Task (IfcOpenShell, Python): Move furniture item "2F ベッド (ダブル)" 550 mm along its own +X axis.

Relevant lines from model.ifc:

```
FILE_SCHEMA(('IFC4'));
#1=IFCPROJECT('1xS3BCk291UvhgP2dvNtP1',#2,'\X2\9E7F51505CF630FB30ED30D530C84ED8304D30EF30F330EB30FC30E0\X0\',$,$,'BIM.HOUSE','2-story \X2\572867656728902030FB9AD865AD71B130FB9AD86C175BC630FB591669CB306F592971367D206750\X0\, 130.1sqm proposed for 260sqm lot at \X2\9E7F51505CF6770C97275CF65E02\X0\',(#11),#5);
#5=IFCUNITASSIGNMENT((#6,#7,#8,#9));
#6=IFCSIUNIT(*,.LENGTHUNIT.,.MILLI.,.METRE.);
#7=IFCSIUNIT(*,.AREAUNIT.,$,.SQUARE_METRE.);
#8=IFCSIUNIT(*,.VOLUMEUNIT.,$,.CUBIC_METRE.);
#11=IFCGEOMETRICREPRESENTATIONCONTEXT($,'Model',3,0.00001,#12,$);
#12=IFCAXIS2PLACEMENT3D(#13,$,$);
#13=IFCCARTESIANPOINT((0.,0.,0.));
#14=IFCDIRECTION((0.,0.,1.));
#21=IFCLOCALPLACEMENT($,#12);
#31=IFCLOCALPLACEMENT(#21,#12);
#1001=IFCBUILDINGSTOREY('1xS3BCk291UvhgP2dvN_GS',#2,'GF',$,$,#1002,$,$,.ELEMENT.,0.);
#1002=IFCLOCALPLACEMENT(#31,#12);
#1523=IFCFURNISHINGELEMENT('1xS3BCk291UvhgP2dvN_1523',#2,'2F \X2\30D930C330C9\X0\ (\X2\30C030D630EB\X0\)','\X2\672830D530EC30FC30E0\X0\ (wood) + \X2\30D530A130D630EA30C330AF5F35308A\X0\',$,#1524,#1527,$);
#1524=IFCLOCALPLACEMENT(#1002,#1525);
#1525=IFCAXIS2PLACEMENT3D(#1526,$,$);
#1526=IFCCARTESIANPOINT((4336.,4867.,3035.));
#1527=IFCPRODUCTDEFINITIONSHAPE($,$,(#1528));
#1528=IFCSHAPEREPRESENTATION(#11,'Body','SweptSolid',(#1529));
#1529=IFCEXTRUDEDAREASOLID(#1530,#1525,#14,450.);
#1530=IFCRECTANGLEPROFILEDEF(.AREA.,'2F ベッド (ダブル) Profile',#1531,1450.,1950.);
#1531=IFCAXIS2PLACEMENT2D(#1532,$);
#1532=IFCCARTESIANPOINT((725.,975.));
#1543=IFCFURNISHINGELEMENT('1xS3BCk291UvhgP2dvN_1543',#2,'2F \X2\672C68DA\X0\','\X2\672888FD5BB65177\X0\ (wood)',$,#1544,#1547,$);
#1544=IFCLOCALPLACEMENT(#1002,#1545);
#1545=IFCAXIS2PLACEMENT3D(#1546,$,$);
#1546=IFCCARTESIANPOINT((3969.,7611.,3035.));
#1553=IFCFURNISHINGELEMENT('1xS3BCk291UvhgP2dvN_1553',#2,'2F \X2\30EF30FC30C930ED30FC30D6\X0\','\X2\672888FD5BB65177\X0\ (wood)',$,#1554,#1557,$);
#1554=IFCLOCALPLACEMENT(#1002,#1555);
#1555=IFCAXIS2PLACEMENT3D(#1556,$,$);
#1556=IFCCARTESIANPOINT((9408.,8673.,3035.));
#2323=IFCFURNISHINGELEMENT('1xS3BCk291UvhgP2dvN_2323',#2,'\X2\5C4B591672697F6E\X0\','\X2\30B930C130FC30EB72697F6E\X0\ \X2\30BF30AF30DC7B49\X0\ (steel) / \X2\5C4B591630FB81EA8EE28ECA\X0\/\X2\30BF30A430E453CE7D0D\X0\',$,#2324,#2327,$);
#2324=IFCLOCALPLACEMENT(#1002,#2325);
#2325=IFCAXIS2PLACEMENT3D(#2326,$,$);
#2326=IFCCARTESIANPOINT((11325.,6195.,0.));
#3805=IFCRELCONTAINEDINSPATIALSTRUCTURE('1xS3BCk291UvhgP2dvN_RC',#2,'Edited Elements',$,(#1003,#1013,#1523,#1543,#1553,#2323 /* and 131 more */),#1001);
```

```python
import ifcopenshell
import ifcopenshell.api.geometry
import ifcopenshell.util.placement

model = ifcopenshell.open("model.ifc")

item = model.by_id(1523)
matrix = ifcopenshell.util.placement.get_local_placement(item.ObjectPlacement)
matrix[:3, 3] += matrix[:3, 0] * 550.0
ifcopenshell.api.geometry.edit_object_placement(model, product=item, matrix=matrix, is_si=False)

print(ifcopenshell.util.placement.get_local_placement(item.ObjectPlacement).round(3) + 0.0)

model.write("model_v2.ifc")
```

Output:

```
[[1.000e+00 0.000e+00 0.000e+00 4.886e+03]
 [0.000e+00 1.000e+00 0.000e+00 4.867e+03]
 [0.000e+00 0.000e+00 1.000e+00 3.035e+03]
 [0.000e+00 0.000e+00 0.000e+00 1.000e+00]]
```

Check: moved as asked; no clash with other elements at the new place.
